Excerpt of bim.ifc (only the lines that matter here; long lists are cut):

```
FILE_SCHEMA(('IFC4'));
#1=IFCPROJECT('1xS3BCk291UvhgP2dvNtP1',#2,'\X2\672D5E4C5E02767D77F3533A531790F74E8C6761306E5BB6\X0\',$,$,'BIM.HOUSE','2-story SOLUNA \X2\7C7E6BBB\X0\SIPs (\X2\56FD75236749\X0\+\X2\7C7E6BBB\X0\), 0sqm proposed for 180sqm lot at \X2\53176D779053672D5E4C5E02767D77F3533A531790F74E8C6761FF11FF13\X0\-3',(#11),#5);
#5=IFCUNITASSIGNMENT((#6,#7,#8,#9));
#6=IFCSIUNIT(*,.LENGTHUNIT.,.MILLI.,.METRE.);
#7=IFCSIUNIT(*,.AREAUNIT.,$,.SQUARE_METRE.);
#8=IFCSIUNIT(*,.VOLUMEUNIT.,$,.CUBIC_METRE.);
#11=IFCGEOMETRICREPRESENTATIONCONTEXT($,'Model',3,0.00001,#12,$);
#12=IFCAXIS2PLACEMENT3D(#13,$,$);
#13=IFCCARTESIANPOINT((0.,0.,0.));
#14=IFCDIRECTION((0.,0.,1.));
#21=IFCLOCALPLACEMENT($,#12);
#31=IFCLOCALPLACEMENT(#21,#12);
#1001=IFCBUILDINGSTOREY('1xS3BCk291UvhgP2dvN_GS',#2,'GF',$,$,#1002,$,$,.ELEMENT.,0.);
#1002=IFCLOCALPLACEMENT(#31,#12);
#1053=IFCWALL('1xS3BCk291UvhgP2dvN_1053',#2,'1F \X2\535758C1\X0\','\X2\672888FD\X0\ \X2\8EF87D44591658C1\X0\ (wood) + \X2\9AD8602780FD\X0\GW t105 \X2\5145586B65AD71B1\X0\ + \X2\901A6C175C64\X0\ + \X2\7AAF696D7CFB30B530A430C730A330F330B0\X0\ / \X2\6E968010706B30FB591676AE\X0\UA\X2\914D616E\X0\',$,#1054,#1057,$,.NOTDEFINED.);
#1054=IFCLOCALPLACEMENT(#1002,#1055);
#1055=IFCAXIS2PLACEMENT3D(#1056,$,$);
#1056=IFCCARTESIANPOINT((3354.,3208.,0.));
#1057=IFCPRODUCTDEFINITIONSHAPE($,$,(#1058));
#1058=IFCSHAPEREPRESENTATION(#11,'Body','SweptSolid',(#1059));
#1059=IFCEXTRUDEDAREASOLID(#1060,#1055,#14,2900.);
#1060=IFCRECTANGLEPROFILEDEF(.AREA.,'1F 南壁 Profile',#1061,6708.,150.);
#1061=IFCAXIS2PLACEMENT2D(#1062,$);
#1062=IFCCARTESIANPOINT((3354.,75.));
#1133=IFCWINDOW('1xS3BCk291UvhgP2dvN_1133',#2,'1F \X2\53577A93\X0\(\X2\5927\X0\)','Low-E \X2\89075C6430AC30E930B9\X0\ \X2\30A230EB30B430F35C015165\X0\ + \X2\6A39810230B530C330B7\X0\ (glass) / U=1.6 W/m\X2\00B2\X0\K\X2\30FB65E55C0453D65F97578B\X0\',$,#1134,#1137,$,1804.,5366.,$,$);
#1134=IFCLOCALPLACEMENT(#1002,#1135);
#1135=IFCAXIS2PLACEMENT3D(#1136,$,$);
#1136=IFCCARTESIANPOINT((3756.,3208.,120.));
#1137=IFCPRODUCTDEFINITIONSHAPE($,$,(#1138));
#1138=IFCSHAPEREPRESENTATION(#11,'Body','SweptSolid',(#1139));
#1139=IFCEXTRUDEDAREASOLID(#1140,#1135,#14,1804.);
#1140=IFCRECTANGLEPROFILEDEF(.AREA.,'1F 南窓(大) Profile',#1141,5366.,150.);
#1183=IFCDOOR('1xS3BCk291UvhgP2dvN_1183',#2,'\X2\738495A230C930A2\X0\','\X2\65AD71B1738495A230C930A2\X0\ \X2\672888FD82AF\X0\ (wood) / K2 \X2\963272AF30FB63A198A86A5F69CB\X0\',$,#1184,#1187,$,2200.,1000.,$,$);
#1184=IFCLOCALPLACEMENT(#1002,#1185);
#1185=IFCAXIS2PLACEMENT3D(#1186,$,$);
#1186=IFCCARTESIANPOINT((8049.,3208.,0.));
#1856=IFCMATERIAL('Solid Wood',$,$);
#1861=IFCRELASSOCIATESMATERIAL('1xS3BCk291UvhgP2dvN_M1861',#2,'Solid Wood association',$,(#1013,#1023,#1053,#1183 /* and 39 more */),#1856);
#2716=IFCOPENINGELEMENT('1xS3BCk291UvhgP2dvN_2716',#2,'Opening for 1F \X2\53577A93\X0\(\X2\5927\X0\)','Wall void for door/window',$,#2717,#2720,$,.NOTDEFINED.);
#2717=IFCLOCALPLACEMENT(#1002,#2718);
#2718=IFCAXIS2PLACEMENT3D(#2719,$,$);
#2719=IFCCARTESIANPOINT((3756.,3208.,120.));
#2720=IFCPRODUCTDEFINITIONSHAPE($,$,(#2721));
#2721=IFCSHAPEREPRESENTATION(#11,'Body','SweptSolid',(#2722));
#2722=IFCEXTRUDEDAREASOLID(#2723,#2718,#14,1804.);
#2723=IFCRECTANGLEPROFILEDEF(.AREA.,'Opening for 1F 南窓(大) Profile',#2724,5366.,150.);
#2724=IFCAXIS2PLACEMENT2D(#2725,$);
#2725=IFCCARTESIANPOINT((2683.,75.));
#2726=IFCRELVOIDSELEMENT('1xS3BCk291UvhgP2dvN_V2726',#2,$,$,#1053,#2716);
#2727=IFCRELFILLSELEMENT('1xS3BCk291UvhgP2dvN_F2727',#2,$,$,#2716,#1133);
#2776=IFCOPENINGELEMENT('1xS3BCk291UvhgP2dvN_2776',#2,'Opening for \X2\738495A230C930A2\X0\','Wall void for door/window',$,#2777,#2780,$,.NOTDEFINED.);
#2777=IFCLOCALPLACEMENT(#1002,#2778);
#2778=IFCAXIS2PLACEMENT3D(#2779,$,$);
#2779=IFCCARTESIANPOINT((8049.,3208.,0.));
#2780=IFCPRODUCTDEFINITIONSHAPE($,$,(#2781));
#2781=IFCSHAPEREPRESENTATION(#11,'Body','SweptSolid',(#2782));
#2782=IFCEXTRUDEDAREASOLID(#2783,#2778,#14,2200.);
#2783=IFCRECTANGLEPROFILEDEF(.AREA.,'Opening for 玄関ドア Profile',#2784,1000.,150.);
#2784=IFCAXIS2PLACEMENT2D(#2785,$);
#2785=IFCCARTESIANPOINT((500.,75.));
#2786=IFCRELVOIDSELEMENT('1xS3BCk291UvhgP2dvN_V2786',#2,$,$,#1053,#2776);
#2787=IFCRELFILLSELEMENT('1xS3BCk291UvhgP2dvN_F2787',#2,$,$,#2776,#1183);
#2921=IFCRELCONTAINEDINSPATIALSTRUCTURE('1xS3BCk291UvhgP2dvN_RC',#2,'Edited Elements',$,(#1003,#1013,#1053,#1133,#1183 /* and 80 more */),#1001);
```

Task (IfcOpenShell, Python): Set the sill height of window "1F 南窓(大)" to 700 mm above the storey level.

```python
import numpy as np
import ifcopenshell
import ifcopenshell.api.geometry
import ifcopenshell.geom
import ifcopenshell.util.element
import ifcopenshell.util.placement
import ifcopenshell.util.shape
import ifcopenshell.util.unit

model = ifcopenshell.open("bim.ifc")
unit_scale = ifcopenshell.util.unit.calculate_unit_scale(model)

window = model.by_id(1133)
opening = window.FillsVoids[0].RelatingOpeningElement
storey = ifcopenshell.util.element.get_container(window, ifc_class="IfcBuildingStorey")
level = ifcopenshell.util.placement.get_local_placement(storey.ObjectPlacement)[2, 3]

# The opening's origin need not be at the sill, so measure its lowest point.
shape = ifcopenshell.geom.create_shape(ifcopenshell.geom.settings(), opening)
bottom = ifcopenshell.util.shape.get_shape_bottom_elevation(shape, shape.geometry) / unit_scale
dz = level + 700.0 - bottom

shift = np.array([0.0, 0.0, dz])
# The window is not placed relative to its opening, so move both.
for product in (opening, window):
    matrix = ifcopenshell.util.placement.get_local_placement(product.ObjectPlacement)
    matrix[:3, 3] += shift
    ifcopenshell.api.geometry.edit_object_placement(model, product=product, matrix=matrix, is_si=False)

print(f"moved by {dz * unit_scale:+.3f} m")

model.write("bim_rev.ifc")
```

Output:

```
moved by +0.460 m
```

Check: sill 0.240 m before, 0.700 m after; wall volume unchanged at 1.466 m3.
